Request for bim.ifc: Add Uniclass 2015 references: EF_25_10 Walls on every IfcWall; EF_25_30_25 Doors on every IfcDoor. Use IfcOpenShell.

First a look at what the model holds.

```python
import ifcopenshell

model = ifcopenshell.open("bim.ifc")
print(model.schema)
print("classifications:", [c.Name for c in model.by_type("IfcClassification")])
for ifc_class in ("IfcDoor", "IfcRoof", "IfcStair", "IfcWall", "IfcWindow"):
    print(ifc_class, len(model.by_type(ifc_class)))
```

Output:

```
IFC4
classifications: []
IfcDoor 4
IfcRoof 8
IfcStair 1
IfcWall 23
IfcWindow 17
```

```python
import ifcopenshell
import ifcopenshell.api.classification

model = ifcopenshell.open("bim.ifc")

system = ifcopenshell.api.classification.add_classification(model, classification="Uniclass 2015")

codes = {
    "IfcWall": ("EF_25_10", "Walls"),
    "IfcDoor": ("EF_25_30_25", "Doors"),
}
for ifc_class, (code, name) in codes.items():
    products = model.by_type(ifc_class)
    ifcopenshell.api.classification.add_reference(
        model, products=products, classification=system, identification=code, name=name
    )
    print(code, len(products))

model.write("bim_edited.ifc")
```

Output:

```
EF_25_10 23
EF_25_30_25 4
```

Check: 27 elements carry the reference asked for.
